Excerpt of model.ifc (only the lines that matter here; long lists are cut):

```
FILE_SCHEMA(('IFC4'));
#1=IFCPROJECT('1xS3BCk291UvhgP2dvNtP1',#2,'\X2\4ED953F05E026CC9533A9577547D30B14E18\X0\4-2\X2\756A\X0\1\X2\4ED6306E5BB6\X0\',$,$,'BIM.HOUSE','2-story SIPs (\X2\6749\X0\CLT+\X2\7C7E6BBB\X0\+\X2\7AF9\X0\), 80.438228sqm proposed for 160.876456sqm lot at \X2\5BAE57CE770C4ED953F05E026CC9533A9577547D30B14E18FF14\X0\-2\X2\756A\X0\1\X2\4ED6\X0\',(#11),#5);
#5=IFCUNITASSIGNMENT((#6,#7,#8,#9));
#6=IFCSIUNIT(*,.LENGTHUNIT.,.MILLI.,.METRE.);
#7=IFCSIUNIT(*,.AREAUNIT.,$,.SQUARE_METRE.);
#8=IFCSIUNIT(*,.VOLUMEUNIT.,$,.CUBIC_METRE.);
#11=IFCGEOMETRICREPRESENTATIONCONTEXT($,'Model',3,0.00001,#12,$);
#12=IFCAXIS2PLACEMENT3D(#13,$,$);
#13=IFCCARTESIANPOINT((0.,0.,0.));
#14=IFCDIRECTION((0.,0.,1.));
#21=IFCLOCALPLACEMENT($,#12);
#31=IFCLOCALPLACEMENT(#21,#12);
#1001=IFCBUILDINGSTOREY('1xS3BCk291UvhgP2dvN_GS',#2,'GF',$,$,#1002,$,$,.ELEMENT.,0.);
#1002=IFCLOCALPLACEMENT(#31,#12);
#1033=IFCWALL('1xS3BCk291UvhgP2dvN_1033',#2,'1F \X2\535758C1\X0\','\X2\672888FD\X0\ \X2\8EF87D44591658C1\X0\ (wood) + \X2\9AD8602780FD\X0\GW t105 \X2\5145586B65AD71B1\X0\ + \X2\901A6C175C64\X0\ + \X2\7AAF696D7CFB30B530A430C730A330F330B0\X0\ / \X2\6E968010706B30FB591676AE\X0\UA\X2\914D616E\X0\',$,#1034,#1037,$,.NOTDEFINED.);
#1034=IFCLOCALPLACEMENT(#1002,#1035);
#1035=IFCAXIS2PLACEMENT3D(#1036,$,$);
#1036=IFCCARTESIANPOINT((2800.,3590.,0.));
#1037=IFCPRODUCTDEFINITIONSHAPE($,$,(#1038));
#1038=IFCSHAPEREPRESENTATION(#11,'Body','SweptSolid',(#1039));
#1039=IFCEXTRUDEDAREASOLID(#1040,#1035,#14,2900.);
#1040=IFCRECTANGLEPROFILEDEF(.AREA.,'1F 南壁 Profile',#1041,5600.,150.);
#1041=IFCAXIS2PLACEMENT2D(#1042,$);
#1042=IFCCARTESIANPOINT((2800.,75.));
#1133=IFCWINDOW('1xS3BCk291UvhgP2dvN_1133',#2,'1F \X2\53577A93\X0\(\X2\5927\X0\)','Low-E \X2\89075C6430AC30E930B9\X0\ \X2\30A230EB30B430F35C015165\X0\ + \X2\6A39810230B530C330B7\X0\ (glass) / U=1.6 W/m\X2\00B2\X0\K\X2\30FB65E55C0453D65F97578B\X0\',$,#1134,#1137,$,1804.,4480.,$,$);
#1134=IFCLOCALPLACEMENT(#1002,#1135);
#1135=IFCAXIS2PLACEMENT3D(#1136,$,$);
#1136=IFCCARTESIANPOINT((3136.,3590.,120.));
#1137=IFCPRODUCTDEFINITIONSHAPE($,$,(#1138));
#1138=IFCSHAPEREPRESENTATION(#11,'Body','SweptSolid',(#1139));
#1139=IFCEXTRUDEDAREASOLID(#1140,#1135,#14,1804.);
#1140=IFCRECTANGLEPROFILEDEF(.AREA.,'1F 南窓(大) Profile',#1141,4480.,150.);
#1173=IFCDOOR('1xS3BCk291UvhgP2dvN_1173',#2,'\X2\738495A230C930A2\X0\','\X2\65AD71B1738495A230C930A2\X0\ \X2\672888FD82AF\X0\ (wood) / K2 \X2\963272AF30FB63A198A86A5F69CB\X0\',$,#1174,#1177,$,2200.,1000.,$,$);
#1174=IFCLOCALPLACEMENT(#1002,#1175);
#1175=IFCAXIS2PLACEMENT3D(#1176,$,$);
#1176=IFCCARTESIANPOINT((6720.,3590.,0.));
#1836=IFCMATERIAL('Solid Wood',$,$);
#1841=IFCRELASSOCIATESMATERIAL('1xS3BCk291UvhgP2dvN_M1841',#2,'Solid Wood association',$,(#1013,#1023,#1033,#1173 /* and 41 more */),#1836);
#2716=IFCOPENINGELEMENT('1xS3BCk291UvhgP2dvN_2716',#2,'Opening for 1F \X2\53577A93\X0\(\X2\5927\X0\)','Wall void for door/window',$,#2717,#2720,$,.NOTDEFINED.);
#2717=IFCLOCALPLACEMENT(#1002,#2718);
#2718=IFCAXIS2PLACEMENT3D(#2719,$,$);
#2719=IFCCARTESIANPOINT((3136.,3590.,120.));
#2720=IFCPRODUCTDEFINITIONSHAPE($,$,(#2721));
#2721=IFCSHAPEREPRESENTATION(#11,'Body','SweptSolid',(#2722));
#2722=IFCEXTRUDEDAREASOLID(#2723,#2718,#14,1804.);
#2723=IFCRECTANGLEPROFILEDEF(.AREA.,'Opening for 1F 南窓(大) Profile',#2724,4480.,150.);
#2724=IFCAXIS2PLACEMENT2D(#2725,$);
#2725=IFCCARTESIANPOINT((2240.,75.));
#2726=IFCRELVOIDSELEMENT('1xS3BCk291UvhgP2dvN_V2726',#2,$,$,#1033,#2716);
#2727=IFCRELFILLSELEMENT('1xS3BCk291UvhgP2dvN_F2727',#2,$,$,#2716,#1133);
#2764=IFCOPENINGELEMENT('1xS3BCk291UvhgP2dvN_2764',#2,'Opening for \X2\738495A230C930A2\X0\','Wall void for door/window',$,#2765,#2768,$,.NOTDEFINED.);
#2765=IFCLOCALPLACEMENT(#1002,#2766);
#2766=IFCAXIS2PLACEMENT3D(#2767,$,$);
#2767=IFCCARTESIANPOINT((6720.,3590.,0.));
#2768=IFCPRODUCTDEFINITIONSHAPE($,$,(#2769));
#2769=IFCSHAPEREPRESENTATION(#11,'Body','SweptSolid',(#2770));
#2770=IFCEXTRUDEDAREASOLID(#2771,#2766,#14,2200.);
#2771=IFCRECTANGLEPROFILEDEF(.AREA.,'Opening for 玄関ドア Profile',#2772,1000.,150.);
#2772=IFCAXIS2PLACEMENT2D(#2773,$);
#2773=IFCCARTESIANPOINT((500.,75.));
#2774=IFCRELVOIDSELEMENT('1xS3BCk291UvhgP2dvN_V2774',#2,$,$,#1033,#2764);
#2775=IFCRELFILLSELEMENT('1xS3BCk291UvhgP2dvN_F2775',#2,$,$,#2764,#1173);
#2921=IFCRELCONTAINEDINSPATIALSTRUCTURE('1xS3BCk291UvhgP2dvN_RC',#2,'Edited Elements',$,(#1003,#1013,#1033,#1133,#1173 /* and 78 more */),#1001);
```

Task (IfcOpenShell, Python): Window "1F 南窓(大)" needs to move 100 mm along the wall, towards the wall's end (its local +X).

```python
import ifcopenshell
import ifcopenshell.api.geometry
import ifcopenshell.util.placement
import ifcopenshell.util.unit

model = ifcopenshell.open("model.ifc")
unit_scale = ifcopenshell.util.unit.calculate_unit_scale(model)

window = model.by_guid("1xS3BCk291UvhgP2dvN_1133")
opening = window.FillsVoids[0].RelatingOpeningElement
wall = opening.VoidsElements[0].RelatingBuildingElement

wall_matrix = ifcopenshell.util.placement.get_local_placement(wall.ObjectPlacement)
shift = wall_matrix[:3, 0] * 0.1 / unit_scale
before = ifcopenshell.util.placement.get_local_placement(window.ObjectPlacement)[:3, 3].copy()

# The window is not placed relative to its opening, so move both.
for product in (opening, window):
    matrix = ifcopenshell.util.placement.get_local_placement(product.ObjectPlacement)
    matrix[:3, 3] += shift
    ifcopenshell.api.geometry.edit_object_placement(model, product=product, matrix=matrix, is_si=False)

after = ifcopenshell.util.placement.get_local_placement(window.ObjectPlacement)[:3, 3]
print("window moved by", (after - before).round(3) + 0.0)

model.write("model-out.ifc")
```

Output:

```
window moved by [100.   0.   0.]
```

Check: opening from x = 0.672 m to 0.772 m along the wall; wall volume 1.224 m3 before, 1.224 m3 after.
